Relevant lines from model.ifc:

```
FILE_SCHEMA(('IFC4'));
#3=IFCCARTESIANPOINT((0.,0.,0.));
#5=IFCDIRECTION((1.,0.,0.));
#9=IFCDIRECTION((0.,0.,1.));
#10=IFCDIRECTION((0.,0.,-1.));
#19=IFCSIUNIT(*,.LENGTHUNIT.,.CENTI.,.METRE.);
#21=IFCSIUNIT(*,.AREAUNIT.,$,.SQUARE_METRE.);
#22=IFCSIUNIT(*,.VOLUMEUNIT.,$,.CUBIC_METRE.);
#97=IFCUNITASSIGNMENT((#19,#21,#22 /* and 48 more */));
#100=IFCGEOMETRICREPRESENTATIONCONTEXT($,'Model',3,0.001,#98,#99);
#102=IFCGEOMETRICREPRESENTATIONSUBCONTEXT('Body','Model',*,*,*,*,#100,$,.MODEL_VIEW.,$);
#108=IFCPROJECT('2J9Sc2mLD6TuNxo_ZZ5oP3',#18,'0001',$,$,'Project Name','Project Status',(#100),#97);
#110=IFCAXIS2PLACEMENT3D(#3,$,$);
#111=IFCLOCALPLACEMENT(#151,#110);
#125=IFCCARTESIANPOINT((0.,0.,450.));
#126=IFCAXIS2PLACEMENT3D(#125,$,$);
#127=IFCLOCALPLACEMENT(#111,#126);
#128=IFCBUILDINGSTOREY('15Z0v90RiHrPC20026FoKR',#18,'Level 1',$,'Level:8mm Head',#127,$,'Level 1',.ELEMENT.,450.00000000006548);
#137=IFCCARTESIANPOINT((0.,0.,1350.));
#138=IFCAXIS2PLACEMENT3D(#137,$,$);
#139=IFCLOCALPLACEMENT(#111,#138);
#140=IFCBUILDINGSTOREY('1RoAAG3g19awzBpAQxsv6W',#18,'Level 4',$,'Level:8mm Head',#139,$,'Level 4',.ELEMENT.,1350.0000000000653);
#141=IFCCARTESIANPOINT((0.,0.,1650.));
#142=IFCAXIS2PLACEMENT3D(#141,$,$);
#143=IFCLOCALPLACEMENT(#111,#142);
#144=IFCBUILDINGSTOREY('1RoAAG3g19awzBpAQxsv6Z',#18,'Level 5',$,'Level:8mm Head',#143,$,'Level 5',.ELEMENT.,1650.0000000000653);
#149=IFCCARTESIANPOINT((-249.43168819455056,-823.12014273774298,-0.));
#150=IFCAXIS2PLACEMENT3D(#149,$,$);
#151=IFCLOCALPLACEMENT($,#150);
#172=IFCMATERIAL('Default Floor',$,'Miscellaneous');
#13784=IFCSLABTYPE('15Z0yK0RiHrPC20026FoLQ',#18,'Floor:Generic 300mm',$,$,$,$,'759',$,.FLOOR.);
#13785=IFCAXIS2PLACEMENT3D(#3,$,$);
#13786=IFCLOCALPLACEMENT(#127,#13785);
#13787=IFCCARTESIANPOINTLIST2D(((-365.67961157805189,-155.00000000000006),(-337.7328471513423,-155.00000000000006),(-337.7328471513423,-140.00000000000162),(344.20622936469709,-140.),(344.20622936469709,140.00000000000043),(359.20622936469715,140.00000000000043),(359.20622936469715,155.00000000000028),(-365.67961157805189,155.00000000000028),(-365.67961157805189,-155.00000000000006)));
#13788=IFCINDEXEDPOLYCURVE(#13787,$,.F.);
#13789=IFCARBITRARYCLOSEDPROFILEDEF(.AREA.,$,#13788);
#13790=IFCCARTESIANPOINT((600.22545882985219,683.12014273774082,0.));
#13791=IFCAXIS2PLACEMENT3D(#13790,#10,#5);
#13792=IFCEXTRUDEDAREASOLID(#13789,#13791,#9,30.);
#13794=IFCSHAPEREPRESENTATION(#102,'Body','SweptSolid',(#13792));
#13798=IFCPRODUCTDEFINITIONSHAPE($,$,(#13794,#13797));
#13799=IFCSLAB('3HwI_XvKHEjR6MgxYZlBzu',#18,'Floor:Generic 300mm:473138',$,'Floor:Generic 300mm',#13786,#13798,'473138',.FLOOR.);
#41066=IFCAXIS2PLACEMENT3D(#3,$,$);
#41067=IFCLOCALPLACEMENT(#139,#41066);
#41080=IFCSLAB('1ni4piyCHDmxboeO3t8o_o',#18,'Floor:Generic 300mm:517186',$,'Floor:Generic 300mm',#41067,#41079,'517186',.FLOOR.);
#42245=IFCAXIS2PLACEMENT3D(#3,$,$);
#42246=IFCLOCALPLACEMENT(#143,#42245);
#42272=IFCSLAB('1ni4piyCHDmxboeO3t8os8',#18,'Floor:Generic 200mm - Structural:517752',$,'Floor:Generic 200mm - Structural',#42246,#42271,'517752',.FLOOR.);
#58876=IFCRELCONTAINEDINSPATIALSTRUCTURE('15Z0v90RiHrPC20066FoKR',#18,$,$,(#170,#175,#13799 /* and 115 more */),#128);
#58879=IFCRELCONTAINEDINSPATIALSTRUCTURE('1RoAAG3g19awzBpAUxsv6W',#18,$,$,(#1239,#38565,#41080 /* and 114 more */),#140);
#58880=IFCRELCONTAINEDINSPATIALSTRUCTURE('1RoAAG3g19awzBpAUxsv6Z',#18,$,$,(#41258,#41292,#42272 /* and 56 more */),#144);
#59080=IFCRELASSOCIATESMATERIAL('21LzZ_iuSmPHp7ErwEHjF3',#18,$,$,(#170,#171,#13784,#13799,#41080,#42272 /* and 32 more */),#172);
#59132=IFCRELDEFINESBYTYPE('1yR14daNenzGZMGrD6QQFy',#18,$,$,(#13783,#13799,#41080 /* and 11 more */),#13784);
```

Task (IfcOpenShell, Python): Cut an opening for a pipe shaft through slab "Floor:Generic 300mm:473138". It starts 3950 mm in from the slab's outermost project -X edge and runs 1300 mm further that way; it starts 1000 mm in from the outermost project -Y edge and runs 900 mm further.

```python
import numpy as np
import ifcopenshell
import ifcopenshell.api.feature
import ifcopenshell.api.geometry
import ifcopenshell.api.root
import ifcopenshell.geom
import ifcopenshell.util.placement
import ifcopenshell.util.representation
import ifcopenshell.util.shape
import ifcopenshell.util.unit

model = ifcopenshell.open("model.ifc")
unit_scale = ifcopenshell.util.unit.calculate_unit_scale(model)
settings = ifcopenshell.geom.settings()


def volume(element):
    """Net volume in cubic metres, openings subtracted."""
    shape = ifcopenshell.geom.create_shape(settings, element)
    return ifcopenshell.util.shape.get_volume(shape.geometry)


slab = model.by_guid("3HwI_XvKHEjR6MgxYZlBzu")
before = volume(slab)

# Extent in the slab's own axes, in metres. The edges named are its -X and -Y sides.
slab_shape = ifcopenshell.geom.create_shape(settings, slab)
vertices = ifcopenshell.util.shape.get_vertices(slab_shape.geometry)
x_min, y_min, bottom = vertices.min(axis=0)
top = vertices[:, 2].max()

opening = ifcopenshell.api.root.create_entity(model, ifc_class="IfcOpeningElement", name="Pipe shaft opening", predefined_type="OPENING")
context = ifcopenshell.util.representation.get_context(model, "Model", "Body", "MODEL_VIEW")
width, depth = 1.3, 0.9
outline = [(0.0, 0.0), (width, 0.0), (width, depth), (0.0, depth), (0.0, 0.0)]
# Overshoot both faces by 50 mm so the cut is clean.
shape = ifcopenshell.api.geometry.add_slab_representation(
    model, context=context, depth=top - bottom + 0.1, polyline=outline
)
ifcopenshell.api.geometry.assign_representation(model, product=opening, representation=shape)

matrix = ifcopenshell.util.placement.get_local_placement(slab.ObjectPlacement)
matrix[:, 3] = matrix @ np.append(np.array([x_min + 3.95, y_min + 1, bottom - 0.05]) / unit_scale, 1.0)
ifcopenshell.api.geometry.edit_object_placement(model, product=opening, matrix=matrix, is_si=False)
ifcopenshell.api.feature.add_feature(model, feature=opening, element=slab)

after = volume(slab)

print(f"slab volume {before:.3f} -> {after:.3f} m3")

model.write("model-out.ifc")
```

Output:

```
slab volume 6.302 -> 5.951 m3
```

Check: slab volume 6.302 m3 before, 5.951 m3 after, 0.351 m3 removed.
